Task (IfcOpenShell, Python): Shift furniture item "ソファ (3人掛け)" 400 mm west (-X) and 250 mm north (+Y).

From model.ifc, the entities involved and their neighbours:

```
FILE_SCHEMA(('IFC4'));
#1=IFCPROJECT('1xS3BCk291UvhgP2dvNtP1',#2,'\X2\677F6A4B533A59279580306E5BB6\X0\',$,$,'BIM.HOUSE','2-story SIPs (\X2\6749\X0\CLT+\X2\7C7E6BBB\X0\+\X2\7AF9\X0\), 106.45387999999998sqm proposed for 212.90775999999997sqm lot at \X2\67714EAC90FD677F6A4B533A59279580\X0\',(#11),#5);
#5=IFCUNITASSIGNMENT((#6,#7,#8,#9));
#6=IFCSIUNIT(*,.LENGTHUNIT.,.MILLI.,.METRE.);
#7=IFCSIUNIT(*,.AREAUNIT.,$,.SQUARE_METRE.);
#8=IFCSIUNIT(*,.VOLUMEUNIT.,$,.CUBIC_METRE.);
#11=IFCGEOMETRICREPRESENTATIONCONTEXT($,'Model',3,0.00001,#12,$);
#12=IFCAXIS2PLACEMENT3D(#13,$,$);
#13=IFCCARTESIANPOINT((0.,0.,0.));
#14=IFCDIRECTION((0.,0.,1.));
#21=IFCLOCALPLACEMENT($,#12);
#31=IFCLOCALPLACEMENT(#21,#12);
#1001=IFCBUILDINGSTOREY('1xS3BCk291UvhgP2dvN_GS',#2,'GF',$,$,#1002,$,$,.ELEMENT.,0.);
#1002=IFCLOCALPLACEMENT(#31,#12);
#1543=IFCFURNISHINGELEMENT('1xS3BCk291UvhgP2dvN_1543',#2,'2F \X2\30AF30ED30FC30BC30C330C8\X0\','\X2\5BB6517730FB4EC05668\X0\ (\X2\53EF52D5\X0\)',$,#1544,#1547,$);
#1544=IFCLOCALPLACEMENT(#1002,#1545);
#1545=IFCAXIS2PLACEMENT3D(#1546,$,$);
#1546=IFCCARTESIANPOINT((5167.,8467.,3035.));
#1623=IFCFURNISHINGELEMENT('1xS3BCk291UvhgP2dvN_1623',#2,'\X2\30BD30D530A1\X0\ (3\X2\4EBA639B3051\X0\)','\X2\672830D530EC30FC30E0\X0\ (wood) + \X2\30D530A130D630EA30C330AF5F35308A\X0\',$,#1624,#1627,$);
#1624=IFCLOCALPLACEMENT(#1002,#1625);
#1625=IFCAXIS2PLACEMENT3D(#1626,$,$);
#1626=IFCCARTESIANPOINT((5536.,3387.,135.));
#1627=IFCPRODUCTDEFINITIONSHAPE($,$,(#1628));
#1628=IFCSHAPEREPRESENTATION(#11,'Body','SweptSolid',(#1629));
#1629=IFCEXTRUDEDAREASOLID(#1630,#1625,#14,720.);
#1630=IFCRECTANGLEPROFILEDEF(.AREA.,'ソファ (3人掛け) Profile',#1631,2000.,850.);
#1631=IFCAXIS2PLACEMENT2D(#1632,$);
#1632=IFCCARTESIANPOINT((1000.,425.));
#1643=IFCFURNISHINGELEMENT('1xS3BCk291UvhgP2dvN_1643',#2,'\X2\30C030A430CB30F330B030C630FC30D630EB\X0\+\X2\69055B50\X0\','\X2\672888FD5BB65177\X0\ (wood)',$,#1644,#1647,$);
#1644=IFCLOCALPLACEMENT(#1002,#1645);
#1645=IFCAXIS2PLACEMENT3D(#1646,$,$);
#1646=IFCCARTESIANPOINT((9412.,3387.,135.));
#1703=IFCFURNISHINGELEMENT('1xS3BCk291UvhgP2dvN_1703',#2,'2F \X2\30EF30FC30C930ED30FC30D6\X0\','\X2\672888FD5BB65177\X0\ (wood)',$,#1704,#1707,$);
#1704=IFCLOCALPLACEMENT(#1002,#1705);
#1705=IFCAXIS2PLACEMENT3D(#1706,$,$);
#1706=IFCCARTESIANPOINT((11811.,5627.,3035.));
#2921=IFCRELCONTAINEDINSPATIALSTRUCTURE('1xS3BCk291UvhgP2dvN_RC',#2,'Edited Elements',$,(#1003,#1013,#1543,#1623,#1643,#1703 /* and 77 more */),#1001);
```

```python
import ifcopenshell
import ifcopenshell.api.geometry
import ifcopenshell.util.placement
import ifcopenshell.util.unit

model = ifcopenshell.open("model.ifc")
unit_scale = ifcopenshell.util.unit.calculate_unit_scale(model)

item = model.by_guid("1xS3BCk291UvhgP2dvN_1623")
matrix = ifcopenshell.util.placement.get_local_placement(item.ObjectPlacement)
matrix[0, 3] -= 0.4 / unit_scale
matrix[1, 3] += 0.25 / unit_scale
ifcopenshell.api.geometry.edit_object_placement(model, product=item, matrix=matrix, is_si=False)

print(ifcopenshell.util.placement.get_local_placement(item.ObjectPlacement).round(3) + 0.0)

model.write("model_v2.ifc")
```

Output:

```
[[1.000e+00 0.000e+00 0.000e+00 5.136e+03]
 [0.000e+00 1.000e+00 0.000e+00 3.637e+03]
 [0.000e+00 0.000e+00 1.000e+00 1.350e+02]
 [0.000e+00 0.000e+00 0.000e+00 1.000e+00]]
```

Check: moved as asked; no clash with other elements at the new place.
